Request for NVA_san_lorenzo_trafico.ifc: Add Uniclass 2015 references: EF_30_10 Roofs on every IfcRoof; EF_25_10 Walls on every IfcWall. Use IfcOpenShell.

First a look at what the model holds.

```python
import ifcopenshell

model = ifcopenshell.open("NVA_san_lorenzo_trafico.ifc")
print(model.schema)
print("classifications:", [c.Name for c in model.by_type("IfcClassification")])
for ifc_class in ("IfcDoor", "IfcRoof", "IfcStair", "IfcWall", "IfcWindow"):
    print(ifc_class, len(model.by_type(ifc_class)))
```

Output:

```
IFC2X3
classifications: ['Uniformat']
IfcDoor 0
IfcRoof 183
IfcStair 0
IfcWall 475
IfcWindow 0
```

```python
import ifcopenshell
import ifcopenshell.api.classification

model = ifcopenshell.open("NVA_san_lorenzo_trafico.ifc")

# IFC2X3 requires Source and Edition and has no link from the project to the system.
system = model.create_entity("IfcClassification", Source="NBS", Edition="2015", Name="Uniclass 2015")

codes = {
    "IfcRoof": ("EF_30_10", "Roofs"),
    "IfcWall": ("EF_25_10", "Walls"),
}
for ifc_class, (code, name) in codes.items():
    products = model.by_type(ifc_class)
    ifcopenshell.api.classification.add_reference(
        model, products=products, classification=system, identification=code, name=name
    )
    print(code, len(products))

model.write("NVA_san_lorenzo_trafico_edited.ifc")
```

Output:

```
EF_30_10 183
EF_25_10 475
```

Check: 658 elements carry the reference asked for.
